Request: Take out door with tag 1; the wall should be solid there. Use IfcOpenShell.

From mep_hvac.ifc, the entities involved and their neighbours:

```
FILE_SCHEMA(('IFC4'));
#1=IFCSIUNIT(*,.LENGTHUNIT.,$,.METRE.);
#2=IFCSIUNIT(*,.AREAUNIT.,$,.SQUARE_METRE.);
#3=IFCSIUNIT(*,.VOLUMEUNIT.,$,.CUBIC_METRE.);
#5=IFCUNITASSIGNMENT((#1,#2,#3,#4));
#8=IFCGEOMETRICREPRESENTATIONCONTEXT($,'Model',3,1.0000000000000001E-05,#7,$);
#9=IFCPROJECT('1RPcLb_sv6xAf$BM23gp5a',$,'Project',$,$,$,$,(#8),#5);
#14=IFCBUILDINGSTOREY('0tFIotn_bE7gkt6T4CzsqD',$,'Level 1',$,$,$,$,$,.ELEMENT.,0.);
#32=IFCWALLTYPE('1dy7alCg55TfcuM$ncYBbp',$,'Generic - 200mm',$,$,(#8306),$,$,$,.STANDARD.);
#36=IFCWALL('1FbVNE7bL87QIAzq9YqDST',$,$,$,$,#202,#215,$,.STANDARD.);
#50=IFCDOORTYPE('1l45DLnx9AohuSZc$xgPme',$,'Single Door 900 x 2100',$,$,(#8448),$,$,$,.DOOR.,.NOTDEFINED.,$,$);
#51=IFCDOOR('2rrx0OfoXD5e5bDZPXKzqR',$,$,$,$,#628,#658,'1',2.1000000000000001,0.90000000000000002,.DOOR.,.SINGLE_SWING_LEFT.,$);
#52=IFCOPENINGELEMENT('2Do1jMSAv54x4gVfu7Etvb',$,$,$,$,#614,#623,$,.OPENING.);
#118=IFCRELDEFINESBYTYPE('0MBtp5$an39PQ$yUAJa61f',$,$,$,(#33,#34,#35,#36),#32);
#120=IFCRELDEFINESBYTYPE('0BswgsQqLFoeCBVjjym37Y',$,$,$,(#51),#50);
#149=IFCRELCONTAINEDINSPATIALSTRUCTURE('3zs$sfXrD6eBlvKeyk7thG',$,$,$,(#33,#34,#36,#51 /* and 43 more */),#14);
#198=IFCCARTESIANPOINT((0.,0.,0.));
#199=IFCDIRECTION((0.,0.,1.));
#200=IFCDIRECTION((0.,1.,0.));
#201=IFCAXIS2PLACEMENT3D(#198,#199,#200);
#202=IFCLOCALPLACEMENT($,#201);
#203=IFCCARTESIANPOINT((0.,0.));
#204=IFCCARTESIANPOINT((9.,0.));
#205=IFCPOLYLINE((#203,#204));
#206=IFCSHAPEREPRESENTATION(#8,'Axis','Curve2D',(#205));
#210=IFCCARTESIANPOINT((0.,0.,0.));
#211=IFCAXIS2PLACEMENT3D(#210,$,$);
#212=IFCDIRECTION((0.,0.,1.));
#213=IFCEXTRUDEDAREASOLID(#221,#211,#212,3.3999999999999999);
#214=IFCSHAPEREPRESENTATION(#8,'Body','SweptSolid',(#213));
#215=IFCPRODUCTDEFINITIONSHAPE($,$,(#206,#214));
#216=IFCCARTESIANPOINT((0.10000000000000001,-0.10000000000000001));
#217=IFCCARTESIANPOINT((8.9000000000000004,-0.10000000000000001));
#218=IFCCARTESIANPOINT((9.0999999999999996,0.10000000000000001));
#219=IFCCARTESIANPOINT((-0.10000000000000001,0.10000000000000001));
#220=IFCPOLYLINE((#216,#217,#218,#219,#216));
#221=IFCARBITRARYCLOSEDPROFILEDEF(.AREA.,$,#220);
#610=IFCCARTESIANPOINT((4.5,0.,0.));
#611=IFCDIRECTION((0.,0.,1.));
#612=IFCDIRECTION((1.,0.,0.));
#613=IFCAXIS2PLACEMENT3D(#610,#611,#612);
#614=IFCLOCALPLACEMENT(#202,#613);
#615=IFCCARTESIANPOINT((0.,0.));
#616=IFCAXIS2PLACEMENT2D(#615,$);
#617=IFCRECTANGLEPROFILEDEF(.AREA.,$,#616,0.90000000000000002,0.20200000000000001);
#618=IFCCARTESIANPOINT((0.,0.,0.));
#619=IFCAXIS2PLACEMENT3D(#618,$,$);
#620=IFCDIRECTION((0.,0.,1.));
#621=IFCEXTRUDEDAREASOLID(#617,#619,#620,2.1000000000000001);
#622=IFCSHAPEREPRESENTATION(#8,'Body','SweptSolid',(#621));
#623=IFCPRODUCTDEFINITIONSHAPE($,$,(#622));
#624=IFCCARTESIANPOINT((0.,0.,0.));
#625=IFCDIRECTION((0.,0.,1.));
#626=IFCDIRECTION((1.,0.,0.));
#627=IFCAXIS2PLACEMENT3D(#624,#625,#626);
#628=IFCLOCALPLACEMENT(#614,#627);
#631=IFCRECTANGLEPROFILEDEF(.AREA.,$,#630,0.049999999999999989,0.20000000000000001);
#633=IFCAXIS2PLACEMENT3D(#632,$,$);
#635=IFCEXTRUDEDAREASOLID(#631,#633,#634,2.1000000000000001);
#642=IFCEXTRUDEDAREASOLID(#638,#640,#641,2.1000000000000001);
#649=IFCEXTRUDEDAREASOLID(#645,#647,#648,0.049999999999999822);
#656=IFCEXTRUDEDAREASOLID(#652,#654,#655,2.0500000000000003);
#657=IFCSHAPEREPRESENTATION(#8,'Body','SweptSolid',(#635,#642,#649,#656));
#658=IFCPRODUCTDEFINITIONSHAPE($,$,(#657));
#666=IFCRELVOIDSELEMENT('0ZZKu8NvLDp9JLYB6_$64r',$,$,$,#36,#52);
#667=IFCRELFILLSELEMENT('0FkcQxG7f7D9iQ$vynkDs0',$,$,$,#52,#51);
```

```python
import ifcopenshell
import ifcopenshell.api.feature
import ifcopenshell.api.root
import ifcopenshell.geom
import ifcopenshell.util.shape

model = ifcopenshell.open("mep_hvac.ifc")
settings = ifcopenshell.geom.settings()


def volume(element):
    """Net volume in cubic metres, openings subtracted."""
    shape = ifcopenshell.geom.create_shape(settings, element)
    return ifcopenshell.util.shape.get_volume(shape.geometry)


door = model.by_guid("2rrx0OfoXD5e5bDZPXKzqR")
opening = door.FillsVoids[0].RelatingOpeningElement
wall = opening.VoidsElements[0].RelatingBuildingElement
before = volume(wall)

ifcopenshell.api.root.remove_product(model, product=door)
ifcopenshell.api.feature.remove_feature(model, feature=opening)

after = volume(wall)

print(f"wall volume {before:.3f} -> {after:.3f} m3")

model.write("mep_hvac_updated.ifc")
```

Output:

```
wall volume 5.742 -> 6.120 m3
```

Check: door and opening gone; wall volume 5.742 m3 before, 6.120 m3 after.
